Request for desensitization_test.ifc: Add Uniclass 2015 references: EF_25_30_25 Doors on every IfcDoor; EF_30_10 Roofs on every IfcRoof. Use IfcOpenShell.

First a look at what the model holds.

```python
import ifcopenshell

model = ifcopenshell.open("desensitization_test.ifc")
print(model.schema)
print("classifications:", [c.Name for c in model.by_type("IfcClassification")])
for ifc_class in ("IfcDoor", "IfcRoof", "IfcStair", "IfcWall", "IfcWindow"):
    print(ifc_class, len(model.by_type(ifc_class)))
```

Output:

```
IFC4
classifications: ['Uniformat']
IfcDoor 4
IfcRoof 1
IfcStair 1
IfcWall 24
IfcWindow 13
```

```python
import ifcopenshell
import ifcopenshell.api.classification

model = ifcopenshell.open("desensitization_test.ifc")

system = ifcopenshell.api.classification.add_classification(model, classification="Uniclass 2015")

codes = {
    "IfcDoor": ("EF_25_30_25", "Doors"),
    "IfcRoof": ("EF_30_10", "Roofs"),
}
for ifc_class, (code, name) in codes.items():
    products = model.by_type(ifc_class)
    ifcopenshell.api.classification.add_reference(
        model, products=products, classification=system, identification=code, name=name
    )
    print(code, len(products))

model.write("desensitization_test_v2.ifc")
```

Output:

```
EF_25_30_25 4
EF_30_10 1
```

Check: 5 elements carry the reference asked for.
